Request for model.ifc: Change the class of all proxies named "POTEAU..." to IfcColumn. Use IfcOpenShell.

First a look at what the model holds.

```python
import re

import ifcopenshell

model = ifcopenshell.open("model.ifc")
print(model.schema)
seen = {}
for e in model.by_type("IfcBuildingElementProxy"):
    name = re.sub(r":\d+(:\d+)?$", "", e.Name or "")  # drop the element id that some exporters append
    seen[name] = seen.get(name, 0) + 1
for name, count in sorted(seen.items()):
    print(count, "x", name)
```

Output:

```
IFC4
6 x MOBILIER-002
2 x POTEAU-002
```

```python
import ifcopenshell
import ifcopenshell.api.root

model = ifcopenshell.open("model.ifc")

proxies = [e.id() for e in model.by_type("IfcBuildingElementProxy") if (e.Name or "").startswith("POTEAU")]
for step_id in proxies:
    proxy = model.by_id(step_id)
    # Reclassifying a typed element also reclassifies its type and the type's other occurrences.
    if proxy.is_a("IfcBuildingElementProxy"):
        ifcopenshell.api.root.reassign_class(model, product=proxy, ifc_class="IfcColumn")

print(sum(model.by_id(i).is_a("IfcColumn") for i in proxies), "reclassified")

model.write("model_rev.ifc")
```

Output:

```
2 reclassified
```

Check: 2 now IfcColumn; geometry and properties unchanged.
